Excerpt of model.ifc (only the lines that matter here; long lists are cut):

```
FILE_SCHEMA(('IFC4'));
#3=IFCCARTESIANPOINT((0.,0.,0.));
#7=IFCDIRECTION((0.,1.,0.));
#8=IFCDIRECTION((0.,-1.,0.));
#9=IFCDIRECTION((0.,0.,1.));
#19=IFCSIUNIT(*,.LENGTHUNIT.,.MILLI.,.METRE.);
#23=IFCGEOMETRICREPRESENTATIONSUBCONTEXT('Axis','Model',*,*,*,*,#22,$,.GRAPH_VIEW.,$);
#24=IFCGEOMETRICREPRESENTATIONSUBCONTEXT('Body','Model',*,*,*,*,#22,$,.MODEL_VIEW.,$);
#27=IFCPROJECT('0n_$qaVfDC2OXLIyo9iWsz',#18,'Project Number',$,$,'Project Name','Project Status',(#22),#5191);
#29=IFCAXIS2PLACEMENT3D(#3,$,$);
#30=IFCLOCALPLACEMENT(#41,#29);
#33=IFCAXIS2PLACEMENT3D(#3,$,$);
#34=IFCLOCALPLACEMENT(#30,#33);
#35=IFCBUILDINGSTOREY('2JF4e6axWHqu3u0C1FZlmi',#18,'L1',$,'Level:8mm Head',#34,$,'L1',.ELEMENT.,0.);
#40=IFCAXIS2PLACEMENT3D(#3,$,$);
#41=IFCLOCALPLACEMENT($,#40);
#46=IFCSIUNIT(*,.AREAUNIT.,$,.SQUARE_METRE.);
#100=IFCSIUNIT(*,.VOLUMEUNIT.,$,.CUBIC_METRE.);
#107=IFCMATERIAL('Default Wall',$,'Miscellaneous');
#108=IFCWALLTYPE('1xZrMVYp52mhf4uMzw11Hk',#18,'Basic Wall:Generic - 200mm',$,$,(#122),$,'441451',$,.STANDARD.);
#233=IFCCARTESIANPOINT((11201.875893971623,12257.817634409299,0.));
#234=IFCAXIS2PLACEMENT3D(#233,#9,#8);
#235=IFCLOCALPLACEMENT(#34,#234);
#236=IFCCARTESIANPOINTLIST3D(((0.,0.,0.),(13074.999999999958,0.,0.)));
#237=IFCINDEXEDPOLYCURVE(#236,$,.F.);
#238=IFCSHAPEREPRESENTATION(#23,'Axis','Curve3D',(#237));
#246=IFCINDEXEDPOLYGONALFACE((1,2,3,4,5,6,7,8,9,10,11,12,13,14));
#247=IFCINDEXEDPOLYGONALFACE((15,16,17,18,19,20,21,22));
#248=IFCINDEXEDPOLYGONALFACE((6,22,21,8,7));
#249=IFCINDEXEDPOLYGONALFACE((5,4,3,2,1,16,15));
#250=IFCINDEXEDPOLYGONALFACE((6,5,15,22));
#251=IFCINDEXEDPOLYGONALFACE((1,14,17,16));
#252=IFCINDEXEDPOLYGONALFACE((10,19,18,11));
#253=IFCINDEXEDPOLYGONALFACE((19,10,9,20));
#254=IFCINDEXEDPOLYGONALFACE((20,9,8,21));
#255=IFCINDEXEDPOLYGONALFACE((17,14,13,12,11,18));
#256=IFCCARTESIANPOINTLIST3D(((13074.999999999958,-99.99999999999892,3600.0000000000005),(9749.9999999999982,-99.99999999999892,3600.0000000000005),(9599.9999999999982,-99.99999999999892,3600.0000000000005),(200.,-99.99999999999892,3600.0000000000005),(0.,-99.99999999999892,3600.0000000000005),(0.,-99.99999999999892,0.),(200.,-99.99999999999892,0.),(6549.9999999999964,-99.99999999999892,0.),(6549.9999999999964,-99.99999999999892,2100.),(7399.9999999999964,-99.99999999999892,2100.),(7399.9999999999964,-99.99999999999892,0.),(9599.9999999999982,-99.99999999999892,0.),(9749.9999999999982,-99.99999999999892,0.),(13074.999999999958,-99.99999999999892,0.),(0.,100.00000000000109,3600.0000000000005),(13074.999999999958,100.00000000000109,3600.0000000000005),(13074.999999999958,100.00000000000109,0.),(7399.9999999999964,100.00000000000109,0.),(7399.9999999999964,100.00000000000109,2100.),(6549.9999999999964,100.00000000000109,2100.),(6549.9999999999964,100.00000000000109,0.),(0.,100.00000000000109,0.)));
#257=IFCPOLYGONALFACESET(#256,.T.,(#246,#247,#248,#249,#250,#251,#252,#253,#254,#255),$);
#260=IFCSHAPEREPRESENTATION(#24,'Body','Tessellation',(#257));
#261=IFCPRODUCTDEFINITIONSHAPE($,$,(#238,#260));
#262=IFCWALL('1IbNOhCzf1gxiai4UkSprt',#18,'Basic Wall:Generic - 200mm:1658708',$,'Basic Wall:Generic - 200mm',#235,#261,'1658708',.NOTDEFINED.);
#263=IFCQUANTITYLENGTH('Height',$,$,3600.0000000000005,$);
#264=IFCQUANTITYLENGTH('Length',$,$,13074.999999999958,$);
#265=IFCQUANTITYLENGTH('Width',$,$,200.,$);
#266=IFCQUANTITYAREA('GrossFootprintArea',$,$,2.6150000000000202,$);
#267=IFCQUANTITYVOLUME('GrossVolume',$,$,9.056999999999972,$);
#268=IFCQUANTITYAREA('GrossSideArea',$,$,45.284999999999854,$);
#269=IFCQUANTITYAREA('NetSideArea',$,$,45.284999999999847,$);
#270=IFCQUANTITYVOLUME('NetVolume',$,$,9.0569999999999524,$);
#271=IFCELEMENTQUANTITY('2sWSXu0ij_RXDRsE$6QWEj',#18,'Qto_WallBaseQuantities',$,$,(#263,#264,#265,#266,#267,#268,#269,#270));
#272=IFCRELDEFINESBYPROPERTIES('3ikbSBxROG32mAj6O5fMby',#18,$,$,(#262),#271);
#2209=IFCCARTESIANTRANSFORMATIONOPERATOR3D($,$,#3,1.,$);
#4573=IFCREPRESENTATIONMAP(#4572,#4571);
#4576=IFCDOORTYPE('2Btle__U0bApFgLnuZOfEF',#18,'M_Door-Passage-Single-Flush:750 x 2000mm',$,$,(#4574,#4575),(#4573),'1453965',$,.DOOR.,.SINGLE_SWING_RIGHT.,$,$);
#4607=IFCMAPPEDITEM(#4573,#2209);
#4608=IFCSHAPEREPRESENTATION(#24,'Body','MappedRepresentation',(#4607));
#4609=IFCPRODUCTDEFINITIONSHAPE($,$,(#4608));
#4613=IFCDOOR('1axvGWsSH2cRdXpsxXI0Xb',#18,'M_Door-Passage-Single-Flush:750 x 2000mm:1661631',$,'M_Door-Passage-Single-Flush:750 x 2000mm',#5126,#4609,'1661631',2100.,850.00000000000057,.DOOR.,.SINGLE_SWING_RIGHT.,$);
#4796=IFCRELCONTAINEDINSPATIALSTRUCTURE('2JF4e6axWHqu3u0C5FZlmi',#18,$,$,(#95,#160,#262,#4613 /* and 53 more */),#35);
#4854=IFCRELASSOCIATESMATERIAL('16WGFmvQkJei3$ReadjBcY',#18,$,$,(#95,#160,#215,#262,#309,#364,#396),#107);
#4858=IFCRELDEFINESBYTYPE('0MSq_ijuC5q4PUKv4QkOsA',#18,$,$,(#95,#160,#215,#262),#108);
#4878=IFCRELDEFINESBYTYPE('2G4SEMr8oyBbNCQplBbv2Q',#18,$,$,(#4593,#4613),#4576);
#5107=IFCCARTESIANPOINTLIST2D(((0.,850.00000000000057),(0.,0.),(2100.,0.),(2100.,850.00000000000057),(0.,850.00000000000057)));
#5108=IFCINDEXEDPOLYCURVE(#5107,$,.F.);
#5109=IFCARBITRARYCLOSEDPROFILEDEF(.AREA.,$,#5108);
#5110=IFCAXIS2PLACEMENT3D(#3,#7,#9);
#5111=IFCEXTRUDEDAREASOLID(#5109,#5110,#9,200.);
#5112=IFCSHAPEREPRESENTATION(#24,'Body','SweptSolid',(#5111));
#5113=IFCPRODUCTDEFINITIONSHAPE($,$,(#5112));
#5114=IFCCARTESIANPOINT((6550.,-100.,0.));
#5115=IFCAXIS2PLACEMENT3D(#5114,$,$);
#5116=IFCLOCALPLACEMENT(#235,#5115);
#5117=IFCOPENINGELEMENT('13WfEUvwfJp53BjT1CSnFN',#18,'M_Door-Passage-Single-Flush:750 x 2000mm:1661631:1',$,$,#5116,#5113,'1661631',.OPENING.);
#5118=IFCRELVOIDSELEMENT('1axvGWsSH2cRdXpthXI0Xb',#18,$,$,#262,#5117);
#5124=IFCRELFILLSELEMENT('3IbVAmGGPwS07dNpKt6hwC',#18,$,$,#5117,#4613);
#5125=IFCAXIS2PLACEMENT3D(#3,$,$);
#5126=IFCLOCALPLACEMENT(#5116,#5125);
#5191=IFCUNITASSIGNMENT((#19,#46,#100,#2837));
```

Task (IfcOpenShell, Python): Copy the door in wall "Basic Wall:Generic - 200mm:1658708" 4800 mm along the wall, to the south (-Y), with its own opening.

```python
import ifcopenshell
import ifcopenshell.api.feature
import ifcopenshell.api.geometry
import ifcopenshell.api.pset
import ifcopenshell.api.root
import ifcopenshell.geom
import ifcopenshell.util.element
import ifcopenshell.util.placement
import ifcopenshell.util.shape
import ifcopenshell.util.unit

model = ifcopenshell.open("model.ifc")
area_scale = ifcopenshell.util.unit.calculate_unit_scale(model, "AREAUNIT")
volume_scale = ifcopenshell.util.unit.calculate_unit_scale(model, "VOLUMEUNIT")
settings = ifcopenshell.geom.settings()


def volume(element):
    """Net volume in cubic metres, openings subtracted."""
    shape = ifcopenshell.geom.create_shape(settings, element)
    return ifcopenshell.util.shape.get_volume(shape.geometry)


def reuse_history(source, copy):
    """copy_class also copies each property set's owner history, people and application; keep the originals."""
    for rel in copy.IsDefinedBy:
        if rel.is_a("IfcRelDefinesByProperties") and (history := rel.RelatingPropertyDefinition.OwnerHistory):
            rel.RelatingPropertyDefinition.OwnerHistory = source.OwnerHistory
            ifcopenshell.util.element.remove_deep2(model, history)


door = model.by_guid("1axvGWsSH2cRdXpsxXI0Xb")
opening = door.FillsVoids[0].RelatingOpeningElement
wall = opening.VoidsElements[0].RelatingBuildingElement
before = volume(wall)
shift = ifcopenshell.util.placement.get_local_placement(wall.ObjectPlacement)[:3, 0] * 4800.0

# copy_class copies the void relationship, type, container and properties, but no geometry.
new_opening = ifcopenshell.api.root.copy_class(model, product=opening)
new_opening.Representation = ifcopenshell.util.element.copy_deep(
    model, opening.Representation, exclude=["IfcGeometricRepresentationContext", "IfcRepresentationMap"]
)
new_opening.Name = "M_Door-Passage-Single-Flush:750 x 2000mm"
new_opening.Tag = None
reuse_history(opening, new_opening)
new_door = ifcopenshell.api.root.copy_class(model, product=door)
new_door.Representation = ifcopenshell.util.element.copy_deep(
    model, door.Representation, exclude=["IfcGeometricRepresentationContext", "IfcRepresentationMap"]
)
new_door.Name = "M_Door-Passage-Single-Flush:750 x 2000mm"
new_door.Tag = None
reuse_history(door, new_door)
ifcopenshell.api.feature.add_filling(model, opening=new_opening, element=new_door)

for old, new in ((opening, new_opening), (door, new_door)):
    matrix = ifcopenshell.util.placement.get_local_placement(old.ObjectPlacement)
    matrix[:3, 3] += shift
    ifcopenshell.api.geometry.edit_object_placement(model, product=new, matrix=matrix, is_si=False)

after = volume(wall)
thickness = 0.2  # wall thickness in metres

# Update the wall's stored quantities.
qto = model.by_id(ifcopenshell.util.element.get_pset(wall, "Qto_WallBaseQuantities", should_inherit=False)["id"])
ifcopenshell.api.pset.edit_qto(model, qto=qto, properties={
    "NetSideArea": after / thickness / area_scale,
    "NetVolume": after / volume_scale,
})

print(f"wall volume {before:.3f} -> {after:.3f} m3")

model.write("model_updated.ifc")
```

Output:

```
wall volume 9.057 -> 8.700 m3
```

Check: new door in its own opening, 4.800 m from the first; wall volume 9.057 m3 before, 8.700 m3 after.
